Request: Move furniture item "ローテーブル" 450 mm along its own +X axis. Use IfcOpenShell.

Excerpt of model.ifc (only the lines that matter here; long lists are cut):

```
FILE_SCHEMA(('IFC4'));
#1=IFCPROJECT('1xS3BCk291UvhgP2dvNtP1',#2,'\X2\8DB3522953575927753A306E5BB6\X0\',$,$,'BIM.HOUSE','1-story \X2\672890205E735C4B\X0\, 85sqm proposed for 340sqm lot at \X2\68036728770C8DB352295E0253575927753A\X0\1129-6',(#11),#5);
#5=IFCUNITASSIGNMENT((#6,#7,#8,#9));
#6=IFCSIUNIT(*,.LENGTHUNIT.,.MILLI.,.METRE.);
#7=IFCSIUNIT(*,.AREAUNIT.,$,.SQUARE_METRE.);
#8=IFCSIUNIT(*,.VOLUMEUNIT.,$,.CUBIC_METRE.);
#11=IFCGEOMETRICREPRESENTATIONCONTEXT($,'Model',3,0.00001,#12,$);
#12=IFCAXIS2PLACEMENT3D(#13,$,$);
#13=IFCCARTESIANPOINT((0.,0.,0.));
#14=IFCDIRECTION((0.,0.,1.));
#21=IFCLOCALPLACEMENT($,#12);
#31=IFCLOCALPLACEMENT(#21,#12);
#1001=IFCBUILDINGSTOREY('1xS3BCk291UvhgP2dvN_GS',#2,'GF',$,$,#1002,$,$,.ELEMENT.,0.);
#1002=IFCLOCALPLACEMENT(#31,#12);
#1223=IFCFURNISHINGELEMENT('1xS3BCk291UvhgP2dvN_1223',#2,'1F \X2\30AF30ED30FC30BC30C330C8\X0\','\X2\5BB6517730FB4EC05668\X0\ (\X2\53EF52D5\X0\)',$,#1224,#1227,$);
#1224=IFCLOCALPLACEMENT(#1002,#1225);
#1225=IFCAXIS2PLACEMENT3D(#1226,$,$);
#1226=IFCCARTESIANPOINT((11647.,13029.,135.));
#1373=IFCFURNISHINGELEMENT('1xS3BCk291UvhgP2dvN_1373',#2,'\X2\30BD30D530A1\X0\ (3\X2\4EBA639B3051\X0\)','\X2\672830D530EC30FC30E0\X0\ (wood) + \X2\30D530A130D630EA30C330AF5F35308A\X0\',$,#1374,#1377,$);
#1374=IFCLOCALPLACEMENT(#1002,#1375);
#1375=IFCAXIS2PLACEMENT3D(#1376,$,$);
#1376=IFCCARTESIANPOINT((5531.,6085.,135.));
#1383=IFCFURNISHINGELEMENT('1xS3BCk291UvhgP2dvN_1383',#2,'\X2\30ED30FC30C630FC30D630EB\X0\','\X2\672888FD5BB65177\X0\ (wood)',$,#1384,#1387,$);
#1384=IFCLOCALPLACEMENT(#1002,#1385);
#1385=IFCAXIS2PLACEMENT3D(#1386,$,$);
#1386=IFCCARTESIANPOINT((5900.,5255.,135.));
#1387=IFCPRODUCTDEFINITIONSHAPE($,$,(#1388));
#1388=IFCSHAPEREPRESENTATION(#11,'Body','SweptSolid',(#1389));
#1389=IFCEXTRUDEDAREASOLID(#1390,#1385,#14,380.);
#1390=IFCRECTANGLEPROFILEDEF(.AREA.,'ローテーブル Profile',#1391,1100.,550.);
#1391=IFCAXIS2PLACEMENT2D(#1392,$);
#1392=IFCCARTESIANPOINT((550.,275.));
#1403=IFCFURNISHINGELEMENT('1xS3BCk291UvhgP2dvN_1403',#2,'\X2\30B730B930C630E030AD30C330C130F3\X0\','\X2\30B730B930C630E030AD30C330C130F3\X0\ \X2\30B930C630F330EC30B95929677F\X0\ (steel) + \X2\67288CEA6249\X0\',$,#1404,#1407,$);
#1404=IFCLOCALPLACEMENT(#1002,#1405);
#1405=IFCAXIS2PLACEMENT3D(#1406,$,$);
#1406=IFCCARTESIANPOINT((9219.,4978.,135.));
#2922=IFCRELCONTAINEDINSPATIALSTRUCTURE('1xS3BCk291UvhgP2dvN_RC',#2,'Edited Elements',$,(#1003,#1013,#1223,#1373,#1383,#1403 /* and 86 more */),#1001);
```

```python
import ifcopenshell
import ifcopenshell.api.geometry
import ifcopenshell.util.placement
import ifcopenshell.util.unit

model = ifcopenshell.open("model.ifc")
unit_scale = ifcopenshell.util.unit.calculate_unit_scale(model)

item = model.by_id(1383)
matrix = ifcopenshell.util.placement.get_local_placement(item.ObjectPlacement)
matrix[:3, 3] += matrix[:3, 0] * 0.45 / unit_scale
ifcopenshell.api.geometry.edit_object_placement(model, product=item, matrix=matrix, is_si=False)

print(ifcopenshell.util.placement.get_local_placement(item.ObjectPlacement).round(3) + 0.0)

model.write("model_rev.ifc")
```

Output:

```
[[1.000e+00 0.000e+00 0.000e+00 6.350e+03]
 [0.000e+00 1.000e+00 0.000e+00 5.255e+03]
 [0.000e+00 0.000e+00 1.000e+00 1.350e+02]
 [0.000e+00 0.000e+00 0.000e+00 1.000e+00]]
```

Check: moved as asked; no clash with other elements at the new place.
